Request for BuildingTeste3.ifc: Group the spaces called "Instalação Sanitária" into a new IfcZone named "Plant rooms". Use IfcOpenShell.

First a look at what the model holds.

```python
import ifcopenshell

model = ifcopenshell.open("BuildingTeste3.ifc")
print(model.schema)
seen = {}
for space in model.by_type("IfcSpace"):
    seen[space.LongName] = seen.get(space.LongName, 0) + 1
for name, count in sorted(seen.items(), key=str):
    print(count, "x", name)
print("zones:", [z.Name for z in model.by_type("IfcZone")][:20])
```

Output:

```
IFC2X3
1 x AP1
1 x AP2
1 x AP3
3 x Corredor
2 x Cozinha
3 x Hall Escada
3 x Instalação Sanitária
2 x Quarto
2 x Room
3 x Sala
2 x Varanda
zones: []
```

```python
import ifcopenshell
import ifcopenshell.api.group
import ifcopenshell.api.root

model = ifcopenshell.open("BuildingTeste3.ifc")

names = {"Instalação Sanitária"}
spaces = [s for s in model.by_type("IfcSpace") if s.LongName in names]

zone = ifcopenshell.api.root.create_entity(model, ifc_class="IfcZone", name="Plant rooms")
ifcopenshell.api.group.assign_group(model, products=spaces, group=zone)
print(len(spaces), "spaces in", zone.Name)

model.write("BuildingTeste3_rev.ifc")
```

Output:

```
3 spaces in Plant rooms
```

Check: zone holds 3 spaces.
